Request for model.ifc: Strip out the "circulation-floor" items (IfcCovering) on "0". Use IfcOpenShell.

First a look at what the model holds.

```python
import ifcopenshell
import ifcopenshell.util.element

model = ifcopenshell.open("model.ifc")
print(model.schema)
storey = next(s for s in model.by_type("IfcBuildingStorey") if s.Name == "0")
coverings = [e for e in ifcopenshell.util.element.get_decomposition(storey) if e.is_a("IfcCovering")]
seen = {}
for e in coverings:
    element_type = ifcopenshell.util.element.get_type(e)
    name = element_type.Name if element_type not in (None, e) else None
    seen[name] = seen.get(name, 0) + 1
for name, count in sorted(seen.items(), key=str):
    print(count, "x", name)
```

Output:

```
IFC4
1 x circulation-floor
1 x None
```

```python
import ifcopenshell
import ifcopenshell.api.root
import ifcopenshell.util.element

model = ifcopenshell.open("model.ifc")

storey = next(s for s in model.by_type("IfcBuildingStorey") if s.Name == "0")
coverings = [e for e in ifcopenshell.util.element.get_decomposition(storey) if e.is_a("IfcCovering")]
targets = [e for e in coverings if (t := ifcopenshell.util.element.get_type(e)) not in (None, e) and t.Name == "circulation-floor"]

for e in targets:
    ifcopenshell.api.root.remove_product(model, product=e)
print(len(targets), "removed")

model.write("model-out.ifc")
```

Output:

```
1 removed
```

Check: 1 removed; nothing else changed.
